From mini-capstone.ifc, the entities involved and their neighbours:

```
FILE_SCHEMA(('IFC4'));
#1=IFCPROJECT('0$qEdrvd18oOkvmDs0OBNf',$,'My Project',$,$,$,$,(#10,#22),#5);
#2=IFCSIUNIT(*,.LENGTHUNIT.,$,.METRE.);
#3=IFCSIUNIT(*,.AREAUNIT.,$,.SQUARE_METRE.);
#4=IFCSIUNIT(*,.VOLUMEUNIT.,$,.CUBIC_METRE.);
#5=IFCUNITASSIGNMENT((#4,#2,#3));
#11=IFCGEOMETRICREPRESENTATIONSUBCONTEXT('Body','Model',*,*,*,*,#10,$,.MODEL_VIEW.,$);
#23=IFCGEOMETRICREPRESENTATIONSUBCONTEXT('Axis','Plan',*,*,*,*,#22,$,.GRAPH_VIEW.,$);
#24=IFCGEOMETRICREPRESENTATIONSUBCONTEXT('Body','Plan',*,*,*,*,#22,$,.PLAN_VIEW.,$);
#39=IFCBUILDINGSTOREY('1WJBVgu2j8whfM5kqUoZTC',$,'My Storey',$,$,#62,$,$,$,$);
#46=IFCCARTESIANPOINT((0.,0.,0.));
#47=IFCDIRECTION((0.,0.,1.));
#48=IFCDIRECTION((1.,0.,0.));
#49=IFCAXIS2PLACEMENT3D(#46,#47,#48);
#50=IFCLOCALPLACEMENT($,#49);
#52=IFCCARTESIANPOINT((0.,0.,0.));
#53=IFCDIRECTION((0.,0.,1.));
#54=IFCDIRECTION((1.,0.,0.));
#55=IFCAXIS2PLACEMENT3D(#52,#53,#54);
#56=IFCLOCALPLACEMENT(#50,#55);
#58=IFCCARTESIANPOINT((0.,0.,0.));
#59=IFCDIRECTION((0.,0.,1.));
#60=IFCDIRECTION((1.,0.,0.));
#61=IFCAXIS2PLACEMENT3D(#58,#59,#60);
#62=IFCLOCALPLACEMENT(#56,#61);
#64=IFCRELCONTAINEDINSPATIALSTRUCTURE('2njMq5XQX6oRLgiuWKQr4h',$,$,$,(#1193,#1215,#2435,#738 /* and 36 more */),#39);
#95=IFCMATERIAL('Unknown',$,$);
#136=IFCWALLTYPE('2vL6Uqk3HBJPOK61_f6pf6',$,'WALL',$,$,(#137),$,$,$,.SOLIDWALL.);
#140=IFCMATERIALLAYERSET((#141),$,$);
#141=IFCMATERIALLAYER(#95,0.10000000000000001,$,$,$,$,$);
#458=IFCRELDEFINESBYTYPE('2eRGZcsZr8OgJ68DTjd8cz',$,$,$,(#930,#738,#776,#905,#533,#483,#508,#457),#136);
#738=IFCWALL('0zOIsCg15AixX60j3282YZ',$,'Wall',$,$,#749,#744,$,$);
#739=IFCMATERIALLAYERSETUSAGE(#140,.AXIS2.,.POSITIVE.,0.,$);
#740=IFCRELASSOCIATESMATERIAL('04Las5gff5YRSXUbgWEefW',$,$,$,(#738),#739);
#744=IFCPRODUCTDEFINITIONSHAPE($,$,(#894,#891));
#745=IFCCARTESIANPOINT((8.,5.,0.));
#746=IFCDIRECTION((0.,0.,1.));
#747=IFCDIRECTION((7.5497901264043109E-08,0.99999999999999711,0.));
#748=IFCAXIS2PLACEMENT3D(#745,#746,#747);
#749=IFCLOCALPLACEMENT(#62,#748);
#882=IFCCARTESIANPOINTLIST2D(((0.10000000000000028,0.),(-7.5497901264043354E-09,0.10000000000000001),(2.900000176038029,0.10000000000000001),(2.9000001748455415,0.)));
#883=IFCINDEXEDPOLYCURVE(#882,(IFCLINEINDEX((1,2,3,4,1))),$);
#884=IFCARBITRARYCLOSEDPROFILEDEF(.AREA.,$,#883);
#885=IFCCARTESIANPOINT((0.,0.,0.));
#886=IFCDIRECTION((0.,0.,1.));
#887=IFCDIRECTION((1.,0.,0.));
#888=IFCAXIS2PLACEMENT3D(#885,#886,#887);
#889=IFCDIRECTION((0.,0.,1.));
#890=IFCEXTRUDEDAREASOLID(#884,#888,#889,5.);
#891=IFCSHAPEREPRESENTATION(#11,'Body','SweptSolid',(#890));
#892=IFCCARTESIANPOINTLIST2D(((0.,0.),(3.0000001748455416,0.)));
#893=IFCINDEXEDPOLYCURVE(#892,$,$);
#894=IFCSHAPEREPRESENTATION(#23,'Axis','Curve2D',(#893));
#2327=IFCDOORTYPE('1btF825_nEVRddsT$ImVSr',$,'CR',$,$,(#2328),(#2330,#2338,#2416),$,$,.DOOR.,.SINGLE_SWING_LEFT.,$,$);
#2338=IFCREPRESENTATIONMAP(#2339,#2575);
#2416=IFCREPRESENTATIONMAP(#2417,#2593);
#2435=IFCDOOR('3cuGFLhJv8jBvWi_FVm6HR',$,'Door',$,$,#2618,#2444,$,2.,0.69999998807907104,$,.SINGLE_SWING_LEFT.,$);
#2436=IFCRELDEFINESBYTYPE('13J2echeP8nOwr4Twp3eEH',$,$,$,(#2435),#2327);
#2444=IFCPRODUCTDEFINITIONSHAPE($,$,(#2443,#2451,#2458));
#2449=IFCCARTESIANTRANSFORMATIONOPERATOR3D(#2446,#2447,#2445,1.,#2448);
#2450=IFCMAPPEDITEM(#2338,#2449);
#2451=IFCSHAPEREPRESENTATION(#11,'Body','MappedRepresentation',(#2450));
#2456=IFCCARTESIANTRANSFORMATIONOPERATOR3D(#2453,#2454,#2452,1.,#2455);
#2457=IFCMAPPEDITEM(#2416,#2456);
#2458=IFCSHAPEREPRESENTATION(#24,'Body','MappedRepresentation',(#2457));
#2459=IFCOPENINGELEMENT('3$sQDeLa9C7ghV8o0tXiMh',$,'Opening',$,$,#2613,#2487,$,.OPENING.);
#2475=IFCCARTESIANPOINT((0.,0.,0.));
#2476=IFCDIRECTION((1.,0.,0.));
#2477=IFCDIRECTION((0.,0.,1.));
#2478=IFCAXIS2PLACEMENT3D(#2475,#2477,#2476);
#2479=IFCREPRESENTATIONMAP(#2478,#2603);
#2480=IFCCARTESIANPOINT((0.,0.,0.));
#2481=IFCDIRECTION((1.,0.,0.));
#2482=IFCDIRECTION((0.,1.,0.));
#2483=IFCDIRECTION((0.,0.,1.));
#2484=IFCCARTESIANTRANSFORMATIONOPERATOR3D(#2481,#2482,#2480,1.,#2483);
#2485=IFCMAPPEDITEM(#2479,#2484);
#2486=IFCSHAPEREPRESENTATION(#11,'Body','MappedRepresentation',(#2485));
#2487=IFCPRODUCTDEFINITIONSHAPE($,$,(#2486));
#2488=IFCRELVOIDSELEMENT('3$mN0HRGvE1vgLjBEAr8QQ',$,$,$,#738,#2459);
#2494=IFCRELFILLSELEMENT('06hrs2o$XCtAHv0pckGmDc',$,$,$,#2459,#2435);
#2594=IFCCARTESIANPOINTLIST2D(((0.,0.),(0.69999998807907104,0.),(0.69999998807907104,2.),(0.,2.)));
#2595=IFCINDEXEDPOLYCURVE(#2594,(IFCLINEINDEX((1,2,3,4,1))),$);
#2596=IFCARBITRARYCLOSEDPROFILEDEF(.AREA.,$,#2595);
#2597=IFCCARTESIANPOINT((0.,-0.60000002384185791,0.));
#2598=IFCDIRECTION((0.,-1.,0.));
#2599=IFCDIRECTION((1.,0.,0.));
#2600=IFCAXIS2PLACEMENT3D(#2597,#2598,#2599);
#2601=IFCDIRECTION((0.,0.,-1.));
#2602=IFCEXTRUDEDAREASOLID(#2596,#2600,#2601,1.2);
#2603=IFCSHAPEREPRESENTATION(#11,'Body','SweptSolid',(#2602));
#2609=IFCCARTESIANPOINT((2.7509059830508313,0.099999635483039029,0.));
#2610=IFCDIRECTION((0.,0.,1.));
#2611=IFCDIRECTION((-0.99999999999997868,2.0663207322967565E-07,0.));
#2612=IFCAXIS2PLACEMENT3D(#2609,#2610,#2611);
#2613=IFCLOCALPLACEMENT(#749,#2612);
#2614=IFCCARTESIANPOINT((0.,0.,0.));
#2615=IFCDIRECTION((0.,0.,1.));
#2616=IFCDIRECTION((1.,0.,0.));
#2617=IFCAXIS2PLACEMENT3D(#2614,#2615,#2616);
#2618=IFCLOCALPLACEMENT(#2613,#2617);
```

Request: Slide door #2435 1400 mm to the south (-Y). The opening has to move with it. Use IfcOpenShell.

```python
import ifcopenshell
import ifcopenshell.api.geometry
import ifcopenshell.util.placement

model = ifcopenshell.open("mini-capstone.ifc")

door = model.by_guid("3cuGFLhJv8jBvWi_FVm6HR")
opening = door.FillsVoids[0].RelatingOpeningElement
wall = opening.VoidsElements[0].RelatingBuildingElement

wall_matrix = ifcopenshell.util.placement.get_local_placement(wall.ObjectPlacement)
shift = wall_matrix[:3, 0] * -1.4
before = ifcopenshell.util.placement.get_local_placement(door.ObjectPlacement)[:3, 3].copy()

# The door is placed relative to its opening, so it follows when the opening moves.
matrix = ifcopenshell.util.placement.get_local_placement(opening.ObjectPlacement)
matrix[:3, 3] += shift
ifcopenshell.api.geometry.edit_object_placement(
    model, product=opening, matrix=matrix, is_si=False, should_transform_children=True
)

after = ifcopenshell.util.placement.get_local_placement(door.ObjectPlacement)[:3, 3]
print("door moved by", (after - before).round(3) + 0.0)

model.write("mini-capstone_rev.ifc")
```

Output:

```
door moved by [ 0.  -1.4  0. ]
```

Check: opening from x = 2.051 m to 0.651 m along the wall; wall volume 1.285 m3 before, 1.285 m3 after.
